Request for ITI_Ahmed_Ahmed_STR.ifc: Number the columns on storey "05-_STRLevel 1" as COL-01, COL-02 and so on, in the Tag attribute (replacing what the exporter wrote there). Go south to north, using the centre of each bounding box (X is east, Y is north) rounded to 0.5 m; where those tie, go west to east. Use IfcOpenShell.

First a look at what the model holds.

```python
import ifcopenshell
import ifcopenshell.util.element
import ifcopenshell.util.placement

model = ifcopenshell.open("ITI_Ahmed_Ahmed_STR.ifc")
print(model.schema)
storey = next(s for s in model.by_type("IfcBuildingStorey") if s.Name == "05-_STRLevel 1")
columns = [e for e in ifcopenshell.util.element.get_decomposition(storey) if e.is_a("IfcColumn")]
for e in sorted(columns, key=lambda e: e.id()):
    origin = ifcopenshell.util.placement.get_local_placement(e.ObjectPlacement)[:3, 3]
    print(e.id(), e.Tag, e.Name, origin.round(2) + 0.0, sep=" | ")
```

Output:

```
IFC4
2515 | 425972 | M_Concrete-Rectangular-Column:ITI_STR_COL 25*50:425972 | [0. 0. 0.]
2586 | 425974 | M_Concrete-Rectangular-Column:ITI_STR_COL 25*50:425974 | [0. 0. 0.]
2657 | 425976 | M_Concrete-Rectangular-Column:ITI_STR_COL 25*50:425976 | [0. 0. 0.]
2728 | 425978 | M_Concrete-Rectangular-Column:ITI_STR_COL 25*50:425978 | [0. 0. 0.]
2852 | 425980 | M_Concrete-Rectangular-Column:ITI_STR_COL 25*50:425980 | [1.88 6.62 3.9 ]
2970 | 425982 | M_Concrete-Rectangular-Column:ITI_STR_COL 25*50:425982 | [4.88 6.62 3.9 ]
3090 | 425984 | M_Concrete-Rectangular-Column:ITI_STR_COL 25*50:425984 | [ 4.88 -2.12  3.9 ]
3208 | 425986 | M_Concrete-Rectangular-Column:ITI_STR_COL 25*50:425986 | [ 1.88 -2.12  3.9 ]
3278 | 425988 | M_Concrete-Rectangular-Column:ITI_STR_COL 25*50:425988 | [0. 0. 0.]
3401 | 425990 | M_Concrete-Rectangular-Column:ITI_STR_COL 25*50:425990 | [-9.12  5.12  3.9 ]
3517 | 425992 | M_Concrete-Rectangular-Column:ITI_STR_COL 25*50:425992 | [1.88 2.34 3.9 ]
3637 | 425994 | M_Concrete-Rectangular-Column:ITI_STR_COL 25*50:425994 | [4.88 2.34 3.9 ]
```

```python
import ifcopenshell
import ifcopenshell.geom
import ifcopenshell.util.element
import ifcopenshell.util.shape

model = ifcopenshell.open("ITI_Ahmed_Ahmed_STR.ifc")
settings = ifcopenshell.geom.settings()
settings.set("use-world-coords", True)


def centre(element):
    shape = ifcopenshell.geom.create_shape(settings, element)
    return ifcopenshell.util.shape.get_bbox_centroid(shape.geometry)


storey = next(s for s in model.by_type("IfcBuildingStorey") if s.Name == "05-_STRLevel 1")
columns = [e for e in ifcopenshell.util.element.get_decomposition(storey) if e.is_a("IfcColumn")]

# Insertion points can sit at a corner or the storey origin, so sort by the geometry (in metres).
centres = {e: centre(e) for e in columns}
columns.sort(key=lambda e: (round(centres[e][1] / 0.5), centres[e][0]))

for i, e in enumerate(columns, start=1):
    number = f"COL-{i:02d}"
    e.Tag = number
    print(e.id(), number)

model.write("ITI_Ahmed_Ahmed_STR-out.ifc")
```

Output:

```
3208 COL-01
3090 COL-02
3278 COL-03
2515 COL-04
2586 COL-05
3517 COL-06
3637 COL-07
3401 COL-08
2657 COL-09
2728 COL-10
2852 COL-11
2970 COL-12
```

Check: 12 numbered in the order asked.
